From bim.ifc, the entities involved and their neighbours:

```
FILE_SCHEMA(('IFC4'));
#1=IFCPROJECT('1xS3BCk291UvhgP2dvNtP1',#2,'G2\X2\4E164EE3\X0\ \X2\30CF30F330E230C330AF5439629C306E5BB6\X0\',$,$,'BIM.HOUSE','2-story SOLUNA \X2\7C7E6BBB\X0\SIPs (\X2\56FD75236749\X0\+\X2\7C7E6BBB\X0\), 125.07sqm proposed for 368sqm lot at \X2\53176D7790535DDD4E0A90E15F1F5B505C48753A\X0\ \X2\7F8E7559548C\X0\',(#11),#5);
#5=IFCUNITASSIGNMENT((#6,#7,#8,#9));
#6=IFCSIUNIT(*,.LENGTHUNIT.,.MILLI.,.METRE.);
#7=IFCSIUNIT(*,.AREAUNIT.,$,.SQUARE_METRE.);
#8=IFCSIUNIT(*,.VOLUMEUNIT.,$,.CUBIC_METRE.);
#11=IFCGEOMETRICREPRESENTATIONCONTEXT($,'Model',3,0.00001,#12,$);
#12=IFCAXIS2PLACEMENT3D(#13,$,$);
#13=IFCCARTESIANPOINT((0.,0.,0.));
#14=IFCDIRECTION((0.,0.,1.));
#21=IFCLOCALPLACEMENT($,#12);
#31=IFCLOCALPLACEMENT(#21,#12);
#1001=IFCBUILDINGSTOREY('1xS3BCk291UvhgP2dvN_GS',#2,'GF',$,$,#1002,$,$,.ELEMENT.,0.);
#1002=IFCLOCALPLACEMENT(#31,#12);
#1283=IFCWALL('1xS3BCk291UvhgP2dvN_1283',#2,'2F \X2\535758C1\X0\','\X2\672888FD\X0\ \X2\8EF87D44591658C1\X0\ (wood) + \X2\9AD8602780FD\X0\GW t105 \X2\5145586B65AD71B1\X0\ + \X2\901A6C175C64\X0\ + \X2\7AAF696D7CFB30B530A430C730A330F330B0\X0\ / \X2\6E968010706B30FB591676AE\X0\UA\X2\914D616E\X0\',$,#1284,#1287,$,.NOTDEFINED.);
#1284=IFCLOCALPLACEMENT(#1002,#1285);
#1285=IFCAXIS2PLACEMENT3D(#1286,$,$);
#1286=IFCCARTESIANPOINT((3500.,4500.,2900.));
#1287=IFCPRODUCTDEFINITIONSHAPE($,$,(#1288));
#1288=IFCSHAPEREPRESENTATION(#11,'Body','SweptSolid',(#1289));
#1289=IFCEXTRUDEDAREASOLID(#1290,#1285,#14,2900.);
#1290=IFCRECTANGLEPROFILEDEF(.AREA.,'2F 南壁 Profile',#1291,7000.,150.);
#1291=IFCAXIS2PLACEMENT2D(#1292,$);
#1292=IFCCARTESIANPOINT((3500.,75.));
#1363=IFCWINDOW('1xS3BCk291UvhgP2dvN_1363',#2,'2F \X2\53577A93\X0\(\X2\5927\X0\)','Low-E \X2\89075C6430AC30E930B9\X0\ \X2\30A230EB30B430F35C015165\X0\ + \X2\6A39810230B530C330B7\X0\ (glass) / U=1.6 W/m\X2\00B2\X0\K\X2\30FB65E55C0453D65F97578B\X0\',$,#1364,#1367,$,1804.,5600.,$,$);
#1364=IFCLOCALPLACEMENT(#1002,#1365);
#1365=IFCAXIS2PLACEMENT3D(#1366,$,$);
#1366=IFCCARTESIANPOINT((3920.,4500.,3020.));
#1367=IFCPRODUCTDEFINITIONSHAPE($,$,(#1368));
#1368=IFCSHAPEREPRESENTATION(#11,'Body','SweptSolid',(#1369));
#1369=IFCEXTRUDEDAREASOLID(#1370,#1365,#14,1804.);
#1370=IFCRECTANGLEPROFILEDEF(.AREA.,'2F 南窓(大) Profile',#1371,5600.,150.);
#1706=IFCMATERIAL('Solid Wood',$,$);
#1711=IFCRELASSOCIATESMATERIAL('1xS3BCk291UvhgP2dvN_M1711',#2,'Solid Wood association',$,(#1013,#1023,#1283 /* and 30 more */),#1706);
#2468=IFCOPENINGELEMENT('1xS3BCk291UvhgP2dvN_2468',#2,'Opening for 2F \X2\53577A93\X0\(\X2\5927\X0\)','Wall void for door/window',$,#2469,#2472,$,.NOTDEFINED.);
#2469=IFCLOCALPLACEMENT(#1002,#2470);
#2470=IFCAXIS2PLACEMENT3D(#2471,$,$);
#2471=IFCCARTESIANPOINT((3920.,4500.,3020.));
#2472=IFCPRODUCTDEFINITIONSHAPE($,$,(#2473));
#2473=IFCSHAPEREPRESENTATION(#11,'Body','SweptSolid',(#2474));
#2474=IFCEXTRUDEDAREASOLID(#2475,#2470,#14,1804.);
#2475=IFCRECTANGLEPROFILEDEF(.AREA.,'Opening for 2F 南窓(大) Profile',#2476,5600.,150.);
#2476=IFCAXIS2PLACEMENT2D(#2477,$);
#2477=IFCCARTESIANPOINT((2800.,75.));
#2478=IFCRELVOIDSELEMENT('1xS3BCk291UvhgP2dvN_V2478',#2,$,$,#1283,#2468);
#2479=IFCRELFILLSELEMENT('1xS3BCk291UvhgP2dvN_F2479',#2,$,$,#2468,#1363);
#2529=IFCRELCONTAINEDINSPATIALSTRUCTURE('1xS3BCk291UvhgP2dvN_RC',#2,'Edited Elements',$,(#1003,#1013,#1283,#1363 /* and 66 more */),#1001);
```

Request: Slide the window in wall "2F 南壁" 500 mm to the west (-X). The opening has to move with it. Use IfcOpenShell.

```python
import ifcopenshell
import ifcopenshell.api.geometry
import ifcopenshell.util.placement

model = ifcopenshell.open("bim.ifc")

window = model.by_guid("1xS3BCk291UvhgP2dvN_1363")
opening = window.FillsVoids[0].RelatingOpeningElement
wall = opening.VoidsElements[0].RelatingBuildingElement

wall_matrix = ifcopenshell.util.placement.get_local_placement(wall.ObjectPlacement)
shift = wall_matrix[:3, 0] * -500.0
before = ifcopenshell.util.placement.get_local_placement(window.ObjectPlacement)[:3, 3].copy()

# The window is not placed relative to its opening, so move both.
for product in (opening, window):
    matrix = ifcopenshell.util.placement.get_local_placement(product.ObjectPlacement)
    matrix[:3, 3] += shift
    ifcopenshell.api.geometry.edit_object_placement(model, product=product, matrix=matrix, is_si=False)

after = ifcopenshell.util.placement.get_local_placement(window.ObjectPlacement)[:3, 3]
print("window moved by", (after - before).round(3) + 0.0)

model.write("bim_v2.ifc")
```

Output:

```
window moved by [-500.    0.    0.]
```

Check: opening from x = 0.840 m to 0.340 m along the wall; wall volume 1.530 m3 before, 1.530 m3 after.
